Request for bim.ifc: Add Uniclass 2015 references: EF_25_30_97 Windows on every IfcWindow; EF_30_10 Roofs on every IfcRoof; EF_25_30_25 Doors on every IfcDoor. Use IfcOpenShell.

First a look at what the model holds.

```python
import ifcopenshell

model = ifcopenshell.open("bim.ifc")
print(model.schema)
print("classifications:", [c.Name for c in model.by_type("IfcClassification")])
for ifc_class in ("IfcDoor", "IfcRoof", "IfcStair", "IfcWall", "IfcWindow"):
    print(ifc_class, len(model.by_type(ifc_class)))
```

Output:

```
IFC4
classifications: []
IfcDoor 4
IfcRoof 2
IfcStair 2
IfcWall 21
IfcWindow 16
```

```python
import ifcopenshell
import ifcopenshell.api.classification

model = ifcopenshell.open("bim.ifc")

system = ifcopenshell.api.classification.add_classification(model, classification="Uniclass 2015")

codes = {
    "IfcWindow": ("EF_25_30_97", "Windows"),
    "IfcRoof": ("EF_30_10", "Roofs"),
    "IfcDoor": ("EF_25_30_25", "Doors"),
}
for ifc_class, (code, name) in codes.items():
    products = model.by_type(ifc_class)
    ifcopenshell.api.classification.add_reference(
        model, products=products, classification=system, identification=code, name=name
    )
    print(code, len(products))

model.write("bim_edited.ifc")
```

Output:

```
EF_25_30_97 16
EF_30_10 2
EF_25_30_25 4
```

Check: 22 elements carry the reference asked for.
